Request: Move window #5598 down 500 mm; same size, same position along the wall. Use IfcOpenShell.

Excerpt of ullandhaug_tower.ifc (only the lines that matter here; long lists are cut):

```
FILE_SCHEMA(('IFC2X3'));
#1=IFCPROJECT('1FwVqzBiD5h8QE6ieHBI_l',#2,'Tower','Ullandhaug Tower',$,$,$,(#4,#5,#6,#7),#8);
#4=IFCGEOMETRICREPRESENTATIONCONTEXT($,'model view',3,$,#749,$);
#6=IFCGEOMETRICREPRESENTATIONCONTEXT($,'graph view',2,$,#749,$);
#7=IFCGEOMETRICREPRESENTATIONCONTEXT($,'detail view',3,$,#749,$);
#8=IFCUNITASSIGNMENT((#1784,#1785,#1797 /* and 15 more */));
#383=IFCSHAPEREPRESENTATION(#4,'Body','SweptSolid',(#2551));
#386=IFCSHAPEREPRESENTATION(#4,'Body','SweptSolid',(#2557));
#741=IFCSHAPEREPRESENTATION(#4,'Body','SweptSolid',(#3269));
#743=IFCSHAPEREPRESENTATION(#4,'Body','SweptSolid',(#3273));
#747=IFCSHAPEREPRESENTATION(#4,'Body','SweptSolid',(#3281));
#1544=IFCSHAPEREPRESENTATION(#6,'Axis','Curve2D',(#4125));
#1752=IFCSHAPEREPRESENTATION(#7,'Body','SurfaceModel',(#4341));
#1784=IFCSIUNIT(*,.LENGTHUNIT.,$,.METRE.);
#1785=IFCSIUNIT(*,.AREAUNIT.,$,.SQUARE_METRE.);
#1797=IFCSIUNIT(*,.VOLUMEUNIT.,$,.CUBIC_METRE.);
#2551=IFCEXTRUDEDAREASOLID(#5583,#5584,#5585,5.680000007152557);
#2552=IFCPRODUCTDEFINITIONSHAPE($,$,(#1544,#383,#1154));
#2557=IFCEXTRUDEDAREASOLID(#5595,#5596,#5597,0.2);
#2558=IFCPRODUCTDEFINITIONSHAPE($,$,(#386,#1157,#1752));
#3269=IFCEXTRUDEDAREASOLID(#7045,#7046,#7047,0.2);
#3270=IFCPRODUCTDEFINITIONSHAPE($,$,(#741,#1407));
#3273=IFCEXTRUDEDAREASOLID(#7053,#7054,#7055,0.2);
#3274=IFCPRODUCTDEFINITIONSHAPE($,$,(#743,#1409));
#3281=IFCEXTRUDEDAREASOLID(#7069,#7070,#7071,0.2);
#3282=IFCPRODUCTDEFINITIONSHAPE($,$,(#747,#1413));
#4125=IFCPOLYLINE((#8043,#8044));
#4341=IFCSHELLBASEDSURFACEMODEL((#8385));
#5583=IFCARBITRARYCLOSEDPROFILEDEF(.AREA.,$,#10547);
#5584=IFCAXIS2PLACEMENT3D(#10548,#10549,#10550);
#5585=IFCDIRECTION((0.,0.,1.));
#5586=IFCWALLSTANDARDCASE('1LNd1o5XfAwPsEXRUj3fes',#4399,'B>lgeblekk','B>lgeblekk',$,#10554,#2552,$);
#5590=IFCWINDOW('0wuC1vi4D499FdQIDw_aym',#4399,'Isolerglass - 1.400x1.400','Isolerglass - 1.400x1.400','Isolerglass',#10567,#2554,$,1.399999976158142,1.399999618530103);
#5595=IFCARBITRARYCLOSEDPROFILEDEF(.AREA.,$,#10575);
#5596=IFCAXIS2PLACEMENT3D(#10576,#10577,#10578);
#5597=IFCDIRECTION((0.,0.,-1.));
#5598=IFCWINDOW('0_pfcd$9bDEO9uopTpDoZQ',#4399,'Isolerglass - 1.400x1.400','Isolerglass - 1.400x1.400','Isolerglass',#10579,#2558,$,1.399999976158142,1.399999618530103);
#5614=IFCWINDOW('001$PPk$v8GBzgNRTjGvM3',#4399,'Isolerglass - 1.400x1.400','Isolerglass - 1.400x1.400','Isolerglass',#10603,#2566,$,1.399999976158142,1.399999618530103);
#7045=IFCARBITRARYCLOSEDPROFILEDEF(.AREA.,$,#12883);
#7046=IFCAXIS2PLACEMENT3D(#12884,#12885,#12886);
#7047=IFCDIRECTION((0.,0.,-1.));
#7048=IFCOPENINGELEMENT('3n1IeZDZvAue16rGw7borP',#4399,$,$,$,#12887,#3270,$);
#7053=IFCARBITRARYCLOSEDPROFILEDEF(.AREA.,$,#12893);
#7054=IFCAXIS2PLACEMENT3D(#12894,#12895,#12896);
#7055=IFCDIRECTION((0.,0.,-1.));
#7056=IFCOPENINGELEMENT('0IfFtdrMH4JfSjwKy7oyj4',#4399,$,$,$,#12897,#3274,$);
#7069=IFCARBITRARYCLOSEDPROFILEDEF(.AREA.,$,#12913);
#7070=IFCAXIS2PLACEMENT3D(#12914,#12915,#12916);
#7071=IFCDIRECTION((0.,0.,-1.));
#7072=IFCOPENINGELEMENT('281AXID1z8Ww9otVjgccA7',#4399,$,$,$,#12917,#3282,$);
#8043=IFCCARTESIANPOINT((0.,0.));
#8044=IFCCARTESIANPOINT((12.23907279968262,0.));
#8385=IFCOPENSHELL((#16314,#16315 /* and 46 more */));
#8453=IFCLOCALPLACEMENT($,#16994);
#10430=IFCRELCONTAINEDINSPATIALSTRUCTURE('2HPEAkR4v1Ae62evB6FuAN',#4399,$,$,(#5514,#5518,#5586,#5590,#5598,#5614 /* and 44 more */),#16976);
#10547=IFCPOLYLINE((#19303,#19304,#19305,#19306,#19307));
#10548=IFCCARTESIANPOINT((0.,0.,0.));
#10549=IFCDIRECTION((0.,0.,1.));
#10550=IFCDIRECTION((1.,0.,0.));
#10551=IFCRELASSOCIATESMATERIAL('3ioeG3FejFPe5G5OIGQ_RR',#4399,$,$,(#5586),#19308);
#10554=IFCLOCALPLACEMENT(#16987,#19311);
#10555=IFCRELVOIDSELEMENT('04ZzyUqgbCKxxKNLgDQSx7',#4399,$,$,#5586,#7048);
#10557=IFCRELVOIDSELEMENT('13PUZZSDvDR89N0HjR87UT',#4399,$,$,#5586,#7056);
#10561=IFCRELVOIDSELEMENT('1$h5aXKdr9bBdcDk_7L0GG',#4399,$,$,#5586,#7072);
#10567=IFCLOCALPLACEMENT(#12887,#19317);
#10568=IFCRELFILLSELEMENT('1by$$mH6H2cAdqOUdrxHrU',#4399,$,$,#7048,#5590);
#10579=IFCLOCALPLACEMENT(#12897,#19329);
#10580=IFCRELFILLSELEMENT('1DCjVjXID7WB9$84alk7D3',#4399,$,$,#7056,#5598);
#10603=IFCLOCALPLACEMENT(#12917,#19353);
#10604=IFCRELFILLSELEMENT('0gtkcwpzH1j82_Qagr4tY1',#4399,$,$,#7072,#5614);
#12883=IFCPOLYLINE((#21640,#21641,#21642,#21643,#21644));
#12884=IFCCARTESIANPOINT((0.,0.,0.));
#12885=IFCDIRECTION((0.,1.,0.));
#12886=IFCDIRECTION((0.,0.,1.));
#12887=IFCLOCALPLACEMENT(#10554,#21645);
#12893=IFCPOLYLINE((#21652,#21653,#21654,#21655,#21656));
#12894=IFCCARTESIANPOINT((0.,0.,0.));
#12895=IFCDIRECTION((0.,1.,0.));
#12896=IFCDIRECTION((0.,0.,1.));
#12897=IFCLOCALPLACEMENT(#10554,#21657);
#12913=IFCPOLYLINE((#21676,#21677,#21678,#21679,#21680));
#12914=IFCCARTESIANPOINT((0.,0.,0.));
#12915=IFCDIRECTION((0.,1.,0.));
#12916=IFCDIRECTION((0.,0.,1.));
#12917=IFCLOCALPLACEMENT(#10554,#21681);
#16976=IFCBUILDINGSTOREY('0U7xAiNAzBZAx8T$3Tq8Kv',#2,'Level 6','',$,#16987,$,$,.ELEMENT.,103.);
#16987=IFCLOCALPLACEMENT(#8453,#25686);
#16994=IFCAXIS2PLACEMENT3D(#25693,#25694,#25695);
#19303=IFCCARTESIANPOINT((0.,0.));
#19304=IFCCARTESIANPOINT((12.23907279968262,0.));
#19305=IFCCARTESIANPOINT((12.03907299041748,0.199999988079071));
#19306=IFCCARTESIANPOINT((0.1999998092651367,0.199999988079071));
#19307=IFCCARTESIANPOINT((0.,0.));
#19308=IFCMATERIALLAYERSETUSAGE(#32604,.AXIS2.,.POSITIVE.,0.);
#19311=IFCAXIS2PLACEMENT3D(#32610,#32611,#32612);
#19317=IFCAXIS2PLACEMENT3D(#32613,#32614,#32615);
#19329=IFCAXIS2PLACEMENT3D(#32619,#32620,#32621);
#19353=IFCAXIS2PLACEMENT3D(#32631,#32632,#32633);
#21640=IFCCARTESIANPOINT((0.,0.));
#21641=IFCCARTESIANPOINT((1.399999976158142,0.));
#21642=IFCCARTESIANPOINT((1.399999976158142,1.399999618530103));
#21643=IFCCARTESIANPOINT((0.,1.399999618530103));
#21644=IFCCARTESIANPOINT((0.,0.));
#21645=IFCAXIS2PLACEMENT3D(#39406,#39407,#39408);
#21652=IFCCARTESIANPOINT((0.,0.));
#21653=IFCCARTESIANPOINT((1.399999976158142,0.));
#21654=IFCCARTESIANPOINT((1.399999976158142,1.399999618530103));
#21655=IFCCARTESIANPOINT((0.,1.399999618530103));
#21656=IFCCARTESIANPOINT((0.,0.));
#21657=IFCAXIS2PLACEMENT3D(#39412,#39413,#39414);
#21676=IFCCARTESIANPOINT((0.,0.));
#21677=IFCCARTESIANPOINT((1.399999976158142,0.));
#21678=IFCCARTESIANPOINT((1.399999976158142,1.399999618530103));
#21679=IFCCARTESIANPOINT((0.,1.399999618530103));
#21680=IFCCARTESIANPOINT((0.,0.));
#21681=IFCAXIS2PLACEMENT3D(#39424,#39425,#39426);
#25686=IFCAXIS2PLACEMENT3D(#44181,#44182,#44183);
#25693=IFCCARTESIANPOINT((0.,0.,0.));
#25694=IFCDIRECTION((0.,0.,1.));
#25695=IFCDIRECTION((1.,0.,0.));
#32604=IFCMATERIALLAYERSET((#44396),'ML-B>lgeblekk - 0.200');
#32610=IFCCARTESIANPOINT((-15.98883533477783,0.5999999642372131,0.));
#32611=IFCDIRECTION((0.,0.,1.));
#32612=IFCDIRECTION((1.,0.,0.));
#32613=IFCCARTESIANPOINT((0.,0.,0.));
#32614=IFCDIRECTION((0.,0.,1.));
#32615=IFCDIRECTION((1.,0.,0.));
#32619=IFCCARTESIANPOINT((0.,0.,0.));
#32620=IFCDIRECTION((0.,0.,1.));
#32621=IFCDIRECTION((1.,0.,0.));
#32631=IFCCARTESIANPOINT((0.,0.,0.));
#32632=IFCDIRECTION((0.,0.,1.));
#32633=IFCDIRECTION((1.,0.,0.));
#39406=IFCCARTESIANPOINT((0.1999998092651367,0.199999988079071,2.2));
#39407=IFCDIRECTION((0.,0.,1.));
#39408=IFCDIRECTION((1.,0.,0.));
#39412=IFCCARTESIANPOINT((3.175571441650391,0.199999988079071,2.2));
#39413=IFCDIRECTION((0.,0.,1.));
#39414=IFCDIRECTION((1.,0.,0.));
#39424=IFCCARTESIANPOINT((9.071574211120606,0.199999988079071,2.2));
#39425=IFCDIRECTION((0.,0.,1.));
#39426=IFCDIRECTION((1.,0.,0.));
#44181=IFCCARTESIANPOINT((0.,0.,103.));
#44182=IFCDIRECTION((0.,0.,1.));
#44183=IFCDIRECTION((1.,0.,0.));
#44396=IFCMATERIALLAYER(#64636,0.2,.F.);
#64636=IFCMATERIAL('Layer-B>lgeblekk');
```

```python
import numpy as np
import ifcopenshell
import ifcopenshell.api.geometry
import ifcopenshell.util.placement
import ifcopenshell.util.unit

model = ifcopenshell.open("ullandhaug_tower.ifc")
unit_scale = ifcopenshell.util.unit.calculate_unit_scale(model)

window = model.by_id(5598)
opening = window.FillsVoids[0].RelatingOpeningElement
dz = -0.5 / unit_scale

shift = np.array([0.0, 0.0, dz])
# The window is placed relative to its opening, so it follows when the opening moves.
matrix = ifcopenshell.util.placement.get_local_placement(opening.ObjectPlacement)
matrix[:3, 3] += shift
ifcopenshell.api.geometry.edit_object_placement(
    model, product=opening, matrix=matrix, is_si=False, should_transform_children=True
)

print(f"moved by {dz * unit_scale:+.3f} m")

model.write("ullandhaug_tower_updated.ifc")
```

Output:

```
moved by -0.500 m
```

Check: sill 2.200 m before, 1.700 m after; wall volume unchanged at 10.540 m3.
